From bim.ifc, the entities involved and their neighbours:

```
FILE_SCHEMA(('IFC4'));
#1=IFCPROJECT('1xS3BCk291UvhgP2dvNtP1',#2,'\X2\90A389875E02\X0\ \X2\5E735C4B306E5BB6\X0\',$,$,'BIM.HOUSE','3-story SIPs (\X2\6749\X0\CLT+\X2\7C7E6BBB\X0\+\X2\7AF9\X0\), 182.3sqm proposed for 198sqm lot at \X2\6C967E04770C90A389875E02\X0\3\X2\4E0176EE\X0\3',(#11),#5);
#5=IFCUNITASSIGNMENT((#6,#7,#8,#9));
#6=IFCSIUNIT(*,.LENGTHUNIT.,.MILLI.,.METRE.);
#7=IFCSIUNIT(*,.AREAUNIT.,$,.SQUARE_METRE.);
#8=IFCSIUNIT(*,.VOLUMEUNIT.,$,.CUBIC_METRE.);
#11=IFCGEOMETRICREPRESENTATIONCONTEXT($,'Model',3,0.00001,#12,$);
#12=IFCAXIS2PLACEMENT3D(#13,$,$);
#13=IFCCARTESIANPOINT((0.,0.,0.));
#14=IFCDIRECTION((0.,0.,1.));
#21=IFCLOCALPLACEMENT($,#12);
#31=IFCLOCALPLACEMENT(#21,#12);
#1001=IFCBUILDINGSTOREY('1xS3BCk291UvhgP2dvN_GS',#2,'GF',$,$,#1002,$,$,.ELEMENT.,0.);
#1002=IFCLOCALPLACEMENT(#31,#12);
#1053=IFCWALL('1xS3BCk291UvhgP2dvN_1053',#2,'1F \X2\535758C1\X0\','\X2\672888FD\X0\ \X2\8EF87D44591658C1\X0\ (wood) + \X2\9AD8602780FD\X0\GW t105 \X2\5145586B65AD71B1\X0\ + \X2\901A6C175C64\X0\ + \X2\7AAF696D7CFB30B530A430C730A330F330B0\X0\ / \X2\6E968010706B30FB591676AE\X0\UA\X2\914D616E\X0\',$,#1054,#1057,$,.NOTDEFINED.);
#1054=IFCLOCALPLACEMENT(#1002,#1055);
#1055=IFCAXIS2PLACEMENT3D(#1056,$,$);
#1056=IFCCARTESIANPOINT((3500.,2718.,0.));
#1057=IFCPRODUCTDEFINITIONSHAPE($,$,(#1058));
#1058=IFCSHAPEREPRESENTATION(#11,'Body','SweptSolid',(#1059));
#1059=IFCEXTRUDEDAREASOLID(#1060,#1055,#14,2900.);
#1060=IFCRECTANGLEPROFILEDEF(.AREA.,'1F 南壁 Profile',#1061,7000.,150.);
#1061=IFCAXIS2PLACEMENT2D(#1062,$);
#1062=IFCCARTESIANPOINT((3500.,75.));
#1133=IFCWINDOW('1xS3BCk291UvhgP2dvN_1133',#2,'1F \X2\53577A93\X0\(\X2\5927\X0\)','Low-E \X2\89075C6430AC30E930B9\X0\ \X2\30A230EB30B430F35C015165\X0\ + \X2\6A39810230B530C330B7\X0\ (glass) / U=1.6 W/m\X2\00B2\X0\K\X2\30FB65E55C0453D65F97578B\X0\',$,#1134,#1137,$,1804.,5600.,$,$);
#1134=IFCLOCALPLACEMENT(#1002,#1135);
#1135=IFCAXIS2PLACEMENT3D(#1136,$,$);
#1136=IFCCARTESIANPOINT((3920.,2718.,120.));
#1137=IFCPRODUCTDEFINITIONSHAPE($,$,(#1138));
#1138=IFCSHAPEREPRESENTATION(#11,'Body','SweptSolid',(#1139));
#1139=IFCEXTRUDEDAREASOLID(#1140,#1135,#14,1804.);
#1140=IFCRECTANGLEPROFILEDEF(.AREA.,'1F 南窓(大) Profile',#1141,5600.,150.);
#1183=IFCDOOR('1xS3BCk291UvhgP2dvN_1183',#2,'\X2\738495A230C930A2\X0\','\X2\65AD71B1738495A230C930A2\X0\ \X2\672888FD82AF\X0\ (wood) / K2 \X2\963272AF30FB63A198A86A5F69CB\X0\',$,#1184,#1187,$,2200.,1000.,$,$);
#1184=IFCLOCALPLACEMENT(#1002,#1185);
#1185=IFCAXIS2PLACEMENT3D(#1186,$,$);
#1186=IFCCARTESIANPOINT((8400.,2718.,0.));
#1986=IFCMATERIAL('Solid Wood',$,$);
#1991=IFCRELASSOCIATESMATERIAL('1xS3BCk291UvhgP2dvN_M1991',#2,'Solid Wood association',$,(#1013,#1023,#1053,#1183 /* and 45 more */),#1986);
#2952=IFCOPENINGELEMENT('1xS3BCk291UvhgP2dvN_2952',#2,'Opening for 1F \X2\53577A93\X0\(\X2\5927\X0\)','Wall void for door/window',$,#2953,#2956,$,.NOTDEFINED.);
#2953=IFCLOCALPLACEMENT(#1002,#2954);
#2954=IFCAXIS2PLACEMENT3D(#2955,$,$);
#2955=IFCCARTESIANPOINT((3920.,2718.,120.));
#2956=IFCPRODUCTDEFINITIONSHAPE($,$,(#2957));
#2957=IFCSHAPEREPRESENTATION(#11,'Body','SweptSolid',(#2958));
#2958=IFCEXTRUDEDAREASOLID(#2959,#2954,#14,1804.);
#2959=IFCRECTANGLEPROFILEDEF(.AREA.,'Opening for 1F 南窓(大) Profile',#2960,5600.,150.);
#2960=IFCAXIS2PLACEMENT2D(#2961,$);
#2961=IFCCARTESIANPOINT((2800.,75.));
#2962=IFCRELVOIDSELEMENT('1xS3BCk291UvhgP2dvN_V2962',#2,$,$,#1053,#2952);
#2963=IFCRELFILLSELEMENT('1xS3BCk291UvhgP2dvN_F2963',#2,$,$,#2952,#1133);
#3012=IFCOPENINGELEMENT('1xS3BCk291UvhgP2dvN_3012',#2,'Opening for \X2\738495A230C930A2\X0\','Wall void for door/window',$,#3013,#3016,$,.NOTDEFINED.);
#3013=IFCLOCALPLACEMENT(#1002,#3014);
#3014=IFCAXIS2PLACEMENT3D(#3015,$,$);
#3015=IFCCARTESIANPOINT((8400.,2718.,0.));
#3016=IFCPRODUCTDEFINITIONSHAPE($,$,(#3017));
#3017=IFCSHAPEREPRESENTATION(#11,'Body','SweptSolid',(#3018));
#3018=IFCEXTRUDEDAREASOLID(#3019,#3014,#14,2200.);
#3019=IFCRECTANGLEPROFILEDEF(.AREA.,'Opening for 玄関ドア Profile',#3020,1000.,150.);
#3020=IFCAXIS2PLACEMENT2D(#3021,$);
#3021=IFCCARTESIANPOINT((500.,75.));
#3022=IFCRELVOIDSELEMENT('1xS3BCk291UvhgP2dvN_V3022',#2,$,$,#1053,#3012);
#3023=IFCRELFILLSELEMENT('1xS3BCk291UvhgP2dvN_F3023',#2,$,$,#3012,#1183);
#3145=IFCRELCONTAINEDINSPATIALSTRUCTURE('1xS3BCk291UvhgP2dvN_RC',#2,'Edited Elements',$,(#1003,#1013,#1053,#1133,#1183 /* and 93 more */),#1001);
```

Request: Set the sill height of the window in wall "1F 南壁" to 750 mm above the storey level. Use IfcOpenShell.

```python
import numpy as np
import ifcopenshell
import ifcopenshell.api.geometry
import ifcopenshell.geom
import ifcopenshell.util.element
import ifcopenshell.util.placement
import ifcopenshell.util.shape
import ifcopenshell.util.unit

model = ifcopenshell.open("bim.ifc")
unit_scale = ifcopenshell.util.unit.calculate_unit_scale(model)

window = model.by_guid("1xS3BCk291UvhgP2dvN_1133")
opening = window.FillsVoids[0].RelatingOpeningElement
storey = ifcopenshell.util.element.get_container(window, ifc_class="IfcBuildingStorey")
level = ifcopenshell.util.placement.get_local_placement(storey.ObjectPlacement)[2, 3]

# The opening's origin need not be at the sill, so measure its lowest point.
shape = ifcopenshell.geom.create_shape(ifcopenshell.geom.settings(), opening)
bottom = ifcopenshell.util.shape.get_shape_bottom_elevation(shape, shape.geometry) / unit_scale
dz = level + 0.75 / unit_scale - bottom

shift = np.array([0.0, 0.0, dz])
# The window is not placed relative to its opening, so move both.
for product in (opening, window):
    matrix = ifcopenshell.util.placement.get_local_placement(product.ObjectPlacement)
    matrix[:3, 3] += shift
    ifcopenshell.api.geometry.edit_object_placement(model, product=product, matrix=matrix, is_si=False)

print(f"moved by {dz * unit_scale:+.3f} m")

model.write("bim_updated.ifc")
```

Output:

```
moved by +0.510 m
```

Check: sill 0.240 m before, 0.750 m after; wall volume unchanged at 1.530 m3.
